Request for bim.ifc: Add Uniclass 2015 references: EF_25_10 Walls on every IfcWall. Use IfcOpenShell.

First a look at what the model holds.

```python
import ifcopenshell

model = ifcopenshell.open("bim.ifc")
print(model.schema)
print("classifications:", [c.Name for c in model.by_type("IfcClassification")])
for ifc_class in ("IfcDoor", "IfcRoof", "IfcStair", "IfcWall", "IfcWindow"):
    print(ifc_class, len(model.by_type(ifc_class)))
```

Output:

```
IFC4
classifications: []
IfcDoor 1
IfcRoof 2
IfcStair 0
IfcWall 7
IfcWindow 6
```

```python
import ifcopenshell
import ifcopenshell.api.classification

model = ifcopenshell.open("bim.ifc")

system = ifcopenshell.api.classification.add_classification(model, classification="Uniclass 2015")

codes = {
    "IfcWall": ("EF_25_10", "Walls"),
}
for ifc_class, (code, name) in codes.items():
    products = model.by_type(ifc_class)
    ifcopenshell.api.classification.add_reference(
        model, products=products, classification=system, identification=code, name=name
    )
    print(code, len(products))

model.write("bim-out.ifc")
```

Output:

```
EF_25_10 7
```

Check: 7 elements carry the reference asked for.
